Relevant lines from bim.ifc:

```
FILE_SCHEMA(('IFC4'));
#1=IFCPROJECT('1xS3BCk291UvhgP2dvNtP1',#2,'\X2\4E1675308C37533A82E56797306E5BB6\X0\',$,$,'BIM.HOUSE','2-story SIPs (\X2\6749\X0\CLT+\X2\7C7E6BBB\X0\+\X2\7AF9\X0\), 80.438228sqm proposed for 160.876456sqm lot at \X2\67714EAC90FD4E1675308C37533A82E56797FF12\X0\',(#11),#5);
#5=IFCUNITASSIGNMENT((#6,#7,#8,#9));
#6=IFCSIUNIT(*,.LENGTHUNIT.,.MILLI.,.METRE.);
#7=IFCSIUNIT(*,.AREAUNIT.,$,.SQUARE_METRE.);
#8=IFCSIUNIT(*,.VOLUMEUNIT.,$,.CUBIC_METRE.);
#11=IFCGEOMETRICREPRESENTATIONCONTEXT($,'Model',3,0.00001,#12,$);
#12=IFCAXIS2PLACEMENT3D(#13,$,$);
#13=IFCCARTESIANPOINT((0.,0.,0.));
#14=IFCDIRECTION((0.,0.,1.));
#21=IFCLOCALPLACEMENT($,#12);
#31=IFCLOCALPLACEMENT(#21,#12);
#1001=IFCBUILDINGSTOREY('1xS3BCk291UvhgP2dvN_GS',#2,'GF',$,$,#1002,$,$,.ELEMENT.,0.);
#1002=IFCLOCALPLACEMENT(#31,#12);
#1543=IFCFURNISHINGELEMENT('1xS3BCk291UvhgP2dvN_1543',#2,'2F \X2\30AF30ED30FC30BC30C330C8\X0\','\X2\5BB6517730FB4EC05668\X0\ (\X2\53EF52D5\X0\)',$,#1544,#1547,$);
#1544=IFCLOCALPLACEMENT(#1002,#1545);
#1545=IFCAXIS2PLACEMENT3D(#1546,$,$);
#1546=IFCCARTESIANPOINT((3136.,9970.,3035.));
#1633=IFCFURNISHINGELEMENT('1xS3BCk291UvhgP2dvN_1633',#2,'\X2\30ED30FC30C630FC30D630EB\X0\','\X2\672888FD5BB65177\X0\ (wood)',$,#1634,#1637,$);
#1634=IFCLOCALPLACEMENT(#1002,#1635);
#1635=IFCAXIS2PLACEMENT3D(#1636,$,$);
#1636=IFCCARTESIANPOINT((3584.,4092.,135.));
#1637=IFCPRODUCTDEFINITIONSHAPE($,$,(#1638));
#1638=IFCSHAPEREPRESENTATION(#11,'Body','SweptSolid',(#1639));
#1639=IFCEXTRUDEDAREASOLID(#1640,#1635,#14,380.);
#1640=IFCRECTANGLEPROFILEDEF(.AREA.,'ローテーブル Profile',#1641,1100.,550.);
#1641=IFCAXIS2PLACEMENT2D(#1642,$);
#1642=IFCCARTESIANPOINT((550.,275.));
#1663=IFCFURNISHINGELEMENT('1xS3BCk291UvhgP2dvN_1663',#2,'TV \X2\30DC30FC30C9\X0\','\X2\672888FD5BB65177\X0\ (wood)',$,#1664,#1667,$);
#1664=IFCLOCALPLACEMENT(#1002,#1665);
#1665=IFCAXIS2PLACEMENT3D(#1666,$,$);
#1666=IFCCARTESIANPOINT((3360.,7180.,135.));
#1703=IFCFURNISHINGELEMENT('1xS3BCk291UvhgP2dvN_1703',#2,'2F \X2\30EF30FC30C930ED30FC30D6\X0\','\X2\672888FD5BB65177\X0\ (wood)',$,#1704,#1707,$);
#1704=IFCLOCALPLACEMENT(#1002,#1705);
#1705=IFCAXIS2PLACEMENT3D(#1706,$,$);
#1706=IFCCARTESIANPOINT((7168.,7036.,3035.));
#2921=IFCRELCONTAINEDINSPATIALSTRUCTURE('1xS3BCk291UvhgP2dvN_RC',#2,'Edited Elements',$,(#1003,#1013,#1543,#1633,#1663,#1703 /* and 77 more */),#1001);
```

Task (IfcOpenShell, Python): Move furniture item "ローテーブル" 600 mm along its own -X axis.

```python
import ifcopenshell
import ifcopenshell.api.geometry
import ifcopenshell.util.placement
import ifcopenshell.util.unit

model = ifcopenshell.open("bim.ifc")
unit_scale = ifcopenshell.util.unit.calculate_unit_scale(model)

item = model.by_guid("1xS3BCk291UvhgP2dvN_1633")
matrix = ifcopenshell.util.placement.get_local_placement(item.ObjectPlacement)
matrix[:3, 3] -= matrix[:3, 0] * 0.6 / unit_scale
ifcopenshell.api.geometry.edit_object_placement(model, product=item, matrix=matrix, is_si=False)

print(ifcopenshell.util.placement.get_local_placement(item.ObjectPlacement).round(3) + 0.0)

model.write("bim_v2.ifc")
```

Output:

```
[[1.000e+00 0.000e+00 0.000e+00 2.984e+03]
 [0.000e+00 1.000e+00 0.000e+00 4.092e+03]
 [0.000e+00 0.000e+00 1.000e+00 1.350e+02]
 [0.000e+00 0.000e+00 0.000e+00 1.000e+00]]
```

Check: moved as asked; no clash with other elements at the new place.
